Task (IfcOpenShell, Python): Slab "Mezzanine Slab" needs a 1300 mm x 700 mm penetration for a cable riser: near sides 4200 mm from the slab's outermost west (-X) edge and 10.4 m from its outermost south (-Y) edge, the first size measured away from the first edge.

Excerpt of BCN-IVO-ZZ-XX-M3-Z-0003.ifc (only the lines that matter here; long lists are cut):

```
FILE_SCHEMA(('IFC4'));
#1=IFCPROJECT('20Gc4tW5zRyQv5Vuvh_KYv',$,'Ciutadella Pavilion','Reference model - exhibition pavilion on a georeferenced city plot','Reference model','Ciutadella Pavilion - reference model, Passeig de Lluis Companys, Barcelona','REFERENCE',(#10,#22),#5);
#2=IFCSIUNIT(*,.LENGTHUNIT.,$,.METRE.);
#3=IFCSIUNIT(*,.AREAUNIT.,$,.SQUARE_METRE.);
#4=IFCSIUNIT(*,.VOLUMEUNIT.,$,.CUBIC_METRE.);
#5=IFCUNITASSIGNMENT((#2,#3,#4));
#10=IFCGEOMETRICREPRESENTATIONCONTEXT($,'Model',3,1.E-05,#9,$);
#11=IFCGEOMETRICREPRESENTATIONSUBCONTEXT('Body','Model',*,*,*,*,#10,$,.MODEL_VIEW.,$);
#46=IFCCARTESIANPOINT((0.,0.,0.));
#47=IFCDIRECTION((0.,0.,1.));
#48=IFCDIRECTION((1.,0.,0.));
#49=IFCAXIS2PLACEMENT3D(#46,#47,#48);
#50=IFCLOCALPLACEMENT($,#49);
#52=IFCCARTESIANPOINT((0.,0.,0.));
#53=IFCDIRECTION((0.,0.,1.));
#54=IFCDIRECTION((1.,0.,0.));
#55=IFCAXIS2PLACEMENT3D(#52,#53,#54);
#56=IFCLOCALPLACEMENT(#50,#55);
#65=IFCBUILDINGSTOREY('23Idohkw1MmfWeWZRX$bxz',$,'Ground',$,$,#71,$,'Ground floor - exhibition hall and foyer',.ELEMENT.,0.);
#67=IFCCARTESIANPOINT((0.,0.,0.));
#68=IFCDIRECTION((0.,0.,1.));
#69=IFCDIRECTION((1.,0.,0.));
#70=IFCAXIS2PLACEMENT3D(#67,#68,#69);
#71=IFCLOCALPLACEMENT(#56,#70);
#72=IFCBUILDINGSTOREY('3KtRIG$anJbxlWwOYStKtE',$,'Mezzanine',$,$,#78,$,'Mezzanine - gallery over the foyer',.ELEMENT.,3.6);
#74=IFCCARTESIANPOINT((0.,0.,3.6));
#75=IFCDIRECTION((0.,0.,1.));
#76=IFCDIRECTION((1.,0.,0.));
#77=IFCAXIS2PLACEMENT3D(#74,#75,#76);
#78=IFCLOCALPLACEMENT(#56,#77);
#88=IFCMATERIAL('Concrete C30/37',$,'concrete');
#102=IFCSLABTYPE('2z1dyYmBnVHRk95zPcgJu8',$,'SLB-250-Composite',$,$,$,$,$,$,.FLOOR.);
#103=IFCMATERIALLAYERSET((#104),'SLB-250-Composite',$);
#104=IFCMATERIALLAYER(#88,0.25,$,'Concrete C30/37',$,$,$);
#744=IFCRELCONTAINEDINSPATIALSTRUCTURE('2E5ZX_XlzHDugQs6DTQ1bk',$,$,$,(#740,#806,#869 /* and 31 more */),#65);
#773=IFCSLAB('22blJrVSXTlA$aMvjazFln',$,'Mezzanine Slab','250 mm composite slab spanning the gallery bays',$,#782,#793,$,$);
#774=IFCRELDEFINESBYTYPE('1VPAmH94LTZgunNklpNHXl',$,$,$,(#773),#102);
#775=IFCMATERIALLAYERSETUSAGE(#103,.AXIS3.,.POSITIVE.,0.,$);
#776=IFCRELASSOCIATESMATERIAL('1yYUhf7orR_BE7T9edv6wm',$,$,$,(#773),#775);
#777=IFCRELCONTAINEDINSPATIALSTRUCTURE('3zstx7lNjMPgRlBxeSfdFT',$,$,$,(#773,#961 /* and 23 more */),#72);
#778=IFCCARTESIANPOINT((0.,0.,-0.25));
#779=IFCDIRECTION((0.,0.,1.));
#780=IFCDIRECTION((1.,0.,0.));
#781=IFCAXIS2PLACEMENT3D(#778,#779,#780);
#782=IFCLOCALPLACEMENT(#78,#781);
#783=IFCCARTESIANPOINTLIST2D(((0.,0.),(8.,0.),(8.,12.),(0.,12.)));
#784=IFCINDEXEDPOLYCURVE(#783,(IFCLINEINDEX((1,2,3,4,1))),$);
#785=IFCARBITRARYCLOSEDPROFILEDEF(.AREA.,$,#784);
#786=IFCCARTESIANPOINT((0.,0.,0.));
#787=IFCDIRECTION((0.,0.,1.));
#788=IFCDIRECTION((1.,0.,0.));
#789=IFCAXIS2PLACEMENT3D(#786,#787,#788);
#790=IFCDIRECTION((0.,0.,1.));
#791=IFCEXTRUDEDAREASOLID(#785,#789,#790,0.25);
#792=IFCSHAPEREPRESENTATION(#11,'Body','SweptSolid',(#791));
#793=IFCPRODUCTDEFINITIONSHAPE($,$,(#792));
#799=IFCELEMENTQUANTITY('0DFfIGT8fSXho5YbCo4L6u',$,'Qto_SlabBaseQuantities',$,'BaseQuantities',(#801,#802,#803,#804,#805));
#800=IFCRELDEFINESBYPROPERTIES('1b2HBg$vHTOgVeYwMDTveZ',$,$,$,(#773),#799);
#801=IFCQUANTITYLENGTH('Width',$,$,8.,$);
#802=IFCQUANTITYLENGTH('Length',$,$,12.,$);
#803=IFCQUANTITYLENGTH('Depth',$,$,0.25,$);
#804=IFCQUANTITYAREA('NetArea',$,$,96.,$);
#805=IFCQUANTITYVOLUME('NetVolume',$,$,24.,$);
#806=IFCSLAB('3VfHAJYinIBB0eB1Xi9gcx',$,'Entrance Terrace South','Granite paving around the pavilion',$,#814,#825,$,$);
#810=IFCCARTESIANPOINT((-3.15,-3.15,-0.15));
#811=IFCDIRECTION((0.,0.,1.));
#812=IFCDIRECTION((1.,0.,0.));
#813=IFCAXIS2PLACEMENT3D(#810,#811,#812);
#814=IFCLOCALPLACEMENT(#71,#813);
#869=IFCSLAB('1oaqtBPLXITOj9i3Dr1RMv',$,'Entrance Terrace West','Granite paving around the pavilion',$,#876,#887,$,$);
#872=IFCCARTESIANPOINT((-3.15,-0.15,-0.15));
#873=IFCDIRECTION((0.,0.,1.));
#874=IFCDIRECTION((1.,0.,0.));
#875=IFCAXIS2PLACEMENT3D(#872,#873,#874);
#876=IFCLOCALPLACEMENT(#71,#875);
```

```python
import numpy as np
import ifcopenshell
import ifcopenshell.api.feature
import ifcopenshell.api.geometry
import ifcopenshell.api.pset
import ifcopenshell.api.root
import ifcopenshell.geom
import ifcopenshell.util.element
import ifcopenshell.util.placement
import ifcopenshell.util.representation
import ifcopenshell.util.shape
import ifcopenshell.util.unit

model = ifcopenshell.open("BCN-IVO-ZZ-XX-M3-Z-0003.ifc")
unit_scale = ifcopenshell.util.unit.calculate_unit_scale(model)
area_scale = ifcopenshell.util.unit.calculate_unit_scale(model, "AREAUNIT")
volume_scale = ifcopenshell.util.unit.calculate_unit_scale(model, "VOLUMEUNIT")
settings = ifcopenshell.geom.settings()


def volume(element):
    """Net volume in cubic metres, openings subtracted."""
    shape = ifcopenshell.geom.create_shape(settings, element)
    return ifcopenshell.util.shape.get_volume(shape.geometry)


slab = model.by_id(773)
before = volume(slab)

# Extent in the slab's own axes, in metres. The edges named are its -X and -Y sides.
slab_shape = ifcopenshell.geom.create_shape(settings, slab)
vertices = ifcopenshell.util.shape.get_vertices(slab_shape.geometry)
x_min, y_min, bottom = vertices.min(axis=0)
top = vertices[:, 2].max()

opening = ifcopenshell.api.root.create_entity(model, ifc_class="IfcOpeningElement", name="Cable riser opening", predefined_type="OPENING")
context = ifcopenshell.util.representation.get_context(model, "Model", "Body", "MODEL_VIEW")
width, depth = 1.3, 0.7
outline = [(0.0, 0.0), (width, 0.0), (width, depth), (0.0, depth), (0.0, 0.0)]
# Overshoot both faces by 50 mm so the cut is clean.
shape = ifcopenshell.api.geometry.add_slab_representation(
    model, context=context, depth=top - bottom + 0.1, polyline=outline
)
ifcopenshell.api.geometry.assign_representation(model, product=opening, representation=shape)

matrix = ifcopenshell.util.placement.get_local_placement(slab.ObjectPlacement)
matrix[:, 3] = matrix @ np.append(np.array([x_min + 4.2, y_min + 10.4, bottom - 0.05]) / unit_scale, 1.0)
ifcopenshell.api.geometry.edit_object_placement(model, product=opening, matrix=matrix, is_si=False)
ifcopenshell.api.feature.add_feature(model, feature=opening, element=slab)

after = volume(slab)

# Update the slab's stored quantities.
qto = model.by_id(ifcopenshell.util.element.get_pset(slab, "Qto_SlabBaseQuantities", should_inherit=False)["id"])
ifcopenshell.api.pset.edit_qto(model, qto=qto, properties={
    "NetArea": after / (top - bottom) / area_scale,
    "NetVolume": after / volume_scale,
})

print(f"slab volume {before:.3f} -> {after:.3f} m3")

model.write("BCN-IVO-ZZ-XX-M3-Z-0003_v2.ifc")
```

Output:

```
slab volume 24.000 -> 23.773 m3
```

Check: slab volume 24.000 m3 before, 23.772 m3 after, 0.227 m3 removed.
